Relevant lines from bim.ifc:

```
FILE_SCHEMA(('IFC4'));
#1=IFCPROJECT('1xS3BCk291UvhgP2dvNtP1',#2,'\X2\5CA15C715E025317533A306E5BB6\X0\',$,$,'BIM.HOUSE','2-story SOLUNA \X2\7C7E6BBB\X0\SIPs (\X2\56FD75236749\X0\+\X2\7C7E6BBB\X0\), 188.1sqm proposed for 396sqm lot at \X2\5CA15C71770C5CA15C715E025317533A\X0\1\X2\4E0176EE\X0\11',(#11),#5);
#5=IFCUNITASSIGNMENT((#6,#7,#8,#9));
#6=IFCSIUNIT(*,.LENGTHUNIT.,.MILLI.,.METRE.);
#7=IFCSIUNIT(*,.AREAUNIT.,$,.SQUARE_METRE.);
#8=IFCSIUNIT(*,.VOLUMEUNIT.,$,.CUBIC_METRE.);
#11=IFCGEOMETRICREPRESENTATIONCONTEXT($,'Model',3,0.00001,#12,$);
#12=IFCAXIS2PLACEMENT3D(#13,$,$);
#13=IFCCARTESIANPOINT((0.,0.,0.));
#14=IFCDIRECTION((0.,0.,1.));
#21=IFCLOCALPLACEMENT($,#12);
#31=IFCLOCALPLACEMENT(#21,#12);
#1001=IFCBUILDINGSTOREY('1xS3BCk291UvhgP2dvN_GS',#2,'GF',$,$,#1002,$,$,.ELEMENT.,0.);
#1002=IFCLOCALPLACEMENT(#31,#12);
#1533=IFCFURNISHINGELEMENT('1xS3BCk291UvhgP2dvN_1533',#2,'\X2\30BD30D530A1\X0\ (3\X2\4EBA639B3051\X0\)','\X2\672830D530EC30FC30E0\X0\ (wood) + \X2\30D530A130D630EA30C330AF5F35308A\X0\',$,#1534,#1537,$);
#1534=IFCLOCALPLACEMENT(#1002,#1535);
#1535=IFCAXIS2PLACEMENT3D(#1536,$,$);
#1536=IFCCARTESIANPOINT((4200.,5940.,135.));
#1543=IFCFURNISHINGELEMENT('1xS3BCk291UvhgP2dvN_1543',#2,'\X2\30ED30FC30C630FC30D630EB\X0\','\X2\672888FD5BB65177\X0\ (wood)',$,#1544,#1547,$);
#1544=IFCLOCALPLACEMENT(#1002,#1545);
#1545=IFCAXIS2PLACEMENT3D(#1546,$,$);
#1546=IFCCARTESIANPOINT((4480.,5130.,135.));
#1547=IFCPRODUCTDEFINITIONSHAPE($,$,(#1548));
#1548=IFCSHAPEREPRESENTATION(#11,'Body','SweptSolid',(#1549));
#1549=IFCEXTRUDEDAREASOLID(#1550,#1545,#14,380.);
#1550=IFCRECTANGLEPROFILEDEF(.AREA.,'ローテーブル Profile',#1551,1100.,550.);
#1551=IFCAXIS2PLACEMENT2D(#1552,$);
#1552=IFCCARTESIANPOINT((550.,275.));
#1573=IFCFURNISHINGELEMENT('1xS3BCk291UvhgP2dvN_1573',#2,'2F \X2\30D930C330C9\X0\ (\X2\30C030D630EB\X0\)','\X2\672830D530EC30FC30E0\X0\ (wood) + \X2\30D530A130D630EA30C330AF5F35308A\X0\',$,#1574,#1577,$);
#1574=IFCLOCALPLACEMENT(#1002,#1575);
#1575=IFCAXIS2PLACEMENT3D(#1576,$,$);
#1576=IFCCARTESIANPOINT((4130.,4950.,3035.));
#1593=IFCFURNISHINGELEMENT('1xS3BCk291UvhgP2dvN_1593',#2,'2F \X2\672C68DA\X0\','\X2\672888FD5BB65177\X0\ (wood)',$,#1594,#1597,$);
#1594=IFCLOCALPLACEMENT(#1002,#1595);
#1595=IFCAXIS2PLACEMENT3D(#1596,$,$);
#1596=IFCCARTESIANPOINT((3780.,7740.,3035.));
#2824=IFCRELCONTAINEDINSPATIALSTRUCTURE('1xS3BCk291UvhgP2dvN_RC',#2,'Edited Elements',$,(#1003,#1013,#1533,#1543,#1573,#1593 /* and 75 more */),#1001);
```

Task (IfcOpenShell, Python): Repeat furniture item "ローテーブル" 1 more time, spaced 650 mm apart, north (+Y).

```python
import numpy as np
import ifcopenshell
import ifcopenshell.api.geometry
import ifcopenshell.api.root
import ifcopenshell.util.element
import ifcopenshell.util.placement
import ifcopenshell.util.unit

model = ifcopenshell.open("bim.ifc")
unit_scale = ifcopenshell.util.unit.calculate_unit_scale(model)


def reuse_history(source, copy):
    """copy_class also copies each property set's owner history, people and application; keep the originals."""
    for rel in copy.IsDefinedBy:
        if rel.is_a("IfcRelDefinesByProperties") and (history := rel.RelatingPropertyDefinition.OwnerHistory):
            rel.RelatingPropertyDefinition.OwnerHistory = source.OwnerHistory
            ifcopenshell.util.element.remove_deep2(model, history)


source = model.by_guid("1xS3BCk291UvhgP2dvN_1543")
base = ifcopenshell.util.placement.get_local_placement(source.ObjectPlacement)
step = np.array([0.0, 1.0, 0.0]) * 0.65 / unit_scale

for i in range(1, 2):
    copy = ifcopenshell.api.root.copy_class(model, product=source)
    copy.Representation = ifcopenshell.util.element.copy_deep(
        model, source.Representation, exclude=["IfcGeometricRepresentationContext", "IfcRepresentationMap"]
    )
    reuse_history(source, copy)
    matrix = base.copy()
    matrix[:3, 3] += i * step
    print("added at", matrix[:3, 3].round(3) + 0.0)
    ifcopenshell.api.geometry.edit_object_placement(model, product=copy, matrix=matrix, is_si=False)

model.write("bim-out.ifc")
```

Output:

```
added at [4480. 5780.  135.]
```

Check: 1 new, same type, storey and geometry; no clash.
